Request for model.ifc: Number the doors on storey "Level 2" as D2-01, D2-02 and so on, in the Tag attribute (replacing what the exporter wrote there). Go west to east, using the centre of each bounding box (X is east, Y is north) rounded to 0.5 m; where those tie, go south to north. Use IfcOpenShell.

First a look at what the model holds.

```python
import ifcopenshell
import ifcopenshell.util.element
import ifcopenshell.util.placement

model = ifcopenshell.open("model.ifc")
print(model.schema)
storey = next(s for s in model.by_type("IfcBuildingStorey") if s.Name == "Level 2")
doors = [e for e in ifcopenshell.util.element.get_decomposition(storey) if e.is_a("IfcDoor")]
for e in sorted(doors, key=lambda e: e.id()):
    origin = ifcopenshell.util.placement.get_local_placement(e.ObjectPlacement)[:3, 3]
    print(e.id(), e.Tag, e.Name, origin.round(2) + 0.0, sep=" | ")
```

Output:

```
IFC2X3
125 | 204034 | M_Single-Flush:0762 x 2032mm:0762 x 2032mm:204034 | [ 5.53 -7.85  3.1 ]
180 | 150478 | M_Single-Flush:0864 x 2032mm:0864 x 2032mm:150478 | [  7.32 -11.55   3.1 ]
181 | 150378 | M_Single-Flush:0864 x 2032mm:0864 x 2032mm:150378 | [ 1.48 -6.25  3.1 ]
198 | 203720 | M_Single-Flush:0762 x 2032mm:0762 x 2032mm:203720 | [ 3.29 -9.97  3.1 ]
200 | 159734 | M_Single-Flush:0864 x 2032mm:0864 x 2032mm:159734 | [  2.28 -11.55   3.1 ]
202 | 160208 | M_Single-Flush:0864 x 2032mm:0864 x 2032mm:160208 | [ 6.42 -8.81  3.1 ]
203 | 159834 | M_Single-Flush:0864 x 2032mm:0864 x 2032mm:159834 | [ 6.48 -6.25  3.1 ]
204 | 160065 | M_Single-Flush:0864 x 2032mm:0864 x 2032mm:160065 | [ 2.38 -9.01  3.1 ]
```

```python
import ifcopenshell
import ifcopenshell.geom
import ifcopenshell.util.element
import ifcopenshell.util.shape

model = ifcopenshell.open("model.ifc")
settings = ifcopenshell.geom.settings()
settings.set("use-world-coords", True)


def centre(element):
    shape = ifcopenshell.geom.create_shape(settings, element)
    return ifcopenshell.util.shape.get_bbox_centroid(shape.geometry)


storey = next(s for s in model.by_type("IfcBuildingStorey") if s.Name == "Level 2")
doors = [e for e in ifcopenshell.util.element.get_decomposition(storey) if e.is_a("IfcDoor")]

# Insertion points can sit at a corner or the storey origin, so sort by the geometry (in metres).
centres = {e: centre(e) for e in doors}
doors.sort(key=lambda e: (round(centres[e][0] / 0.5), centres[e][1]))

for i, e in enumerate(doors, start=1):
    number = f"D2-{i:02d}"
    e.Tag = number
    print(e.id(), number)

model.write("model_updated.ifc")
```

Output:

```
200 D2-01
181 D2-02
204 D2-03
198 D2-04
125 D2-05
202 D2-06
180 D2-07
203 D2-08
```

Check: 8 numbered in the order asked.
